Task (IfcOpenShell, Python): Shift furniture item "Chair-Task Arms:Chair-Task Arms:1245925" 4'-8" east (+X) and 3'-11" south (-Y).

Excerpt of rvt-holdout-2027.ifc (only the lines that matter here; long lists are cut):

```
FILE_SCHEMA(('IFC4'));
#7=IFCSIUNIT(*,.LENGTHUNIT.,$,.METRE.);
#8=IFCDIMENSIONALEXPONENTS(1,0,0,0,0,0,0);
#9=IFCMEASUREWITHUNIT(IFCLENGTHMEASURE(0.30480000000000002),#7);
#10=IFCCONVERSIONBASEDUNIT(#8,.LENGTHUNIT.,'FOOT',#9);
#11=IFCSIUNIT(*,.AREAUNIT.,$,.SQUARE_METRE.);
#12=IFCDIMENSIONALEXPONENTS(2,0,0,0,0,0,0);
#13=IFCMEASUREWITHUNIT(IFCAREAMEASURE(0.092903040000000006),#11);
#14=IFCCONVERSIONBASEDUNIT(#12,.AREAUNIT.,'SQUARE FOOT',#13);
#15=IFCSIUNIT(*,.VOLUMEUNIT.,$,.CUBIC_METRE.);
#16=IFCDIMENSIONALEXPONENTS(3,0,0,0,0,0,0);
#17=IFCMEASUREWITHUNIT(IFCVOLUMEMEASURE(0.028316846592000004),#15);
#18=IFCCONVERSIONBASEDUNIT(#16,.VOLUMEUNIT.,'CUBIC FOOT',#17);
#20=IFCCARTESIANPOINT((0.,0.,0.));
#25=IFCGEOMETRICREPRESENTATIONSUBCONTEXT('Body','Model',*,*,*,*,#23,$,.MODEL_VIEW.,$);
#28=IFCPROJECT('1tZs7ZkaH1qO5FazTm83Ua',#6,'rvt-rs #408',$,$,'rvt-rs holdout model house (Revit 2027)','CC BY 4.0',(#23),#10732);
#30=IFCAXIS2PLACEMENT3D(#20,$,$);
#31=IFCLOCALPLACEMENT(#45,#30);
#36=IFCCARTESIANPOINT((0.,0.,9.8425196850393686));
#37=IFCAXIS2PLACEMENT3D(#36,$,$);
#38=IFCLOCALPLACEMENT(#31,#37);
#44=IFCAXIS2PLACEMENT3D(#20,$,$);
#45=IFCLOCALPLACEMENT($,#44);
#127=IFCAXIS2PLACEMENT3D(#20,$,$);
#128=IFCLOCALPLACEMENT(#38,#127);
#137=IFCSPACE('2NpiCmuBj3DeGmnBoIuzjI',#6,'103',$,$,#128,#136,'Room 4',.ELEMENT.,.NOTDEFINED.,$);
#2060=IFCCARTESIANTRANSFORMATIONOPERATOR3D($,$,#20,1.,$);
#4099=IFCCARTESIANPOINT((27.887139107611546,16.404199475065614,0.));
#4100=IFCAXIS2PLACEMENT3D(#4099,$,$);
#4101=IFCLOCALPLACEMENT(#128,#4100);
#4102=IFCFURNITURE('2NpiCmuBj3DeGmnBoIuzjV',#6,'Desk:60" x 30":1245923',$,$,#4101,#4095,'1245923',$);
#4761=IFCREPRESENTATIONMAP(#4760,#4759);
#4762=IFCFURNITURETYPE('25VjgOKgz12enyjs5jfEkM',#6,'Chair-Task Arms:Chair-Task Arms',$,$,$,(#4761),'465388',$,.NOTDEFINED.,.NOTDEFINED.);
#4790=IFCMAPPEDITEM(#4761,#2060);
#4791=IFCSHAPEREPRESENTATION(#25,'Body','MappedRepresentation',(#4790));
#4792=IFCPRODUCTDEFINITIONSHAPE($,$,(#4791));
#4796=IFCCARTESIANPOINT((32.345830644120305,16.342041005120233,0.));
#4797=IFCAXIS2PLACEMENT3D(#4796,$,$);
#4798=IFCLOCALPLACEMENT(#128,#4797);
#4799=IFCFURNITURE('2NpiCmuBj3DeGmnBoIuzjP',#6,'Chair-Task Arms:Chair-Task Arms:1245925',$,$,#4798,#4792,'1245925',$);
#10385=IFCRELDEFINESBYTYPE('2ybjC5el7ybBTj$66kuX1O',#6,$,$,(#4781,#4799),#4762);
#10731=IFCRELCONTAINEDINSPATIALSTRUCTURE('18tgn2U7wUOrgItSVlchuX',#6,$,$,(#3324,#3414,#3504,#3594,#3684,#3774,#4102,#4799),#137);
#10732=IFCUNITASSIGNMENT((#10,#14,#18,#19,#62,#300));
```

```python
import ifcopenshell
import ifcopenshell.api.geometry
import ifcopenshell.util.placement
import ifcopenshell.util.unit

model = ifcopenshell.open("rvt-holdout-2027.ifc")
unit_scale = ifcopenshell.util.unit.calculate_unit_scale(model)

item = model.by_guid("2NpiCmuBj3DeGmnBoIuzjP")
matrix = ifcopenshell.util.placement.get_local_placement(item.ObjectPlacement)
matrix[0, 3] += 56 * 0.0254 / unit_scale
matrix[1, 3] -= 47 * 0.0254 / unit_scale
ifcopenshell.api.geometry.edit_object_placement(model, product=item, matrix=matrix, is_si=False)

print(ifcopenshell.util.placement.get_local_placement(item.ObjectPlacement).round(3) + 0.0)

model.write("rvt-holdout-2027_rev.ifc")
```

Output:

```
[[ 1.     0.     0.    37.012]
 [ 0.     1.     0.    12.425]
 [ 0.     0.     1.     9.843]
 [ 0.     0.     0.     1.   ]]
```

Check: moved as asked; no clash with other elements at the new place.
